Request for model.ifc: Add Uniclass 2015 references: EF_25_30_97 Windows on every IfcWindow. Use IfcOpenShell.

First a look at what the model holds.

```python
import ifcopenshell

model = ifcopenshell.open("model.ifc")
print(model.schema)
print("classifications:", [c.Name for c in model.by_type("IfcClassification")])
for ifc_class in ("IfcDoor", "IfcRoof", "IfcStair", "IfcWall", "IfcWindow"):
    print(ifc_class, len(model.by_type(ifc_class)))
```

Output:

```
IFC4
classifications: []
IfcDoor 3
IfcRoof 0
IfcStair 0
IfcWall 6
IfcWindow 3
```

```python
import ifcopenshell
import ifcopenshell.api.classification

model = ifcopenshell.open("model.ifc")

system = ifcopenshell.api.classification.add_classification(model, classification="Uniclass 2015")

codes = {
    "IfcWindow": ("EF_25_30_97", "Windows"),
}
for ifc_class, (code, name) in codes.items():
    products = model.by_type(ifc_class)
    ifcopenshell.api.classification.add_reference(
        model, products=products, classification=system, identification=code, name=name
    )
    print(code, len(products))

model.write("model_updated.ifc")
```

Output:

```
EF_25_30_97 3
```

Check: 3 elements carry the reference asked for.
